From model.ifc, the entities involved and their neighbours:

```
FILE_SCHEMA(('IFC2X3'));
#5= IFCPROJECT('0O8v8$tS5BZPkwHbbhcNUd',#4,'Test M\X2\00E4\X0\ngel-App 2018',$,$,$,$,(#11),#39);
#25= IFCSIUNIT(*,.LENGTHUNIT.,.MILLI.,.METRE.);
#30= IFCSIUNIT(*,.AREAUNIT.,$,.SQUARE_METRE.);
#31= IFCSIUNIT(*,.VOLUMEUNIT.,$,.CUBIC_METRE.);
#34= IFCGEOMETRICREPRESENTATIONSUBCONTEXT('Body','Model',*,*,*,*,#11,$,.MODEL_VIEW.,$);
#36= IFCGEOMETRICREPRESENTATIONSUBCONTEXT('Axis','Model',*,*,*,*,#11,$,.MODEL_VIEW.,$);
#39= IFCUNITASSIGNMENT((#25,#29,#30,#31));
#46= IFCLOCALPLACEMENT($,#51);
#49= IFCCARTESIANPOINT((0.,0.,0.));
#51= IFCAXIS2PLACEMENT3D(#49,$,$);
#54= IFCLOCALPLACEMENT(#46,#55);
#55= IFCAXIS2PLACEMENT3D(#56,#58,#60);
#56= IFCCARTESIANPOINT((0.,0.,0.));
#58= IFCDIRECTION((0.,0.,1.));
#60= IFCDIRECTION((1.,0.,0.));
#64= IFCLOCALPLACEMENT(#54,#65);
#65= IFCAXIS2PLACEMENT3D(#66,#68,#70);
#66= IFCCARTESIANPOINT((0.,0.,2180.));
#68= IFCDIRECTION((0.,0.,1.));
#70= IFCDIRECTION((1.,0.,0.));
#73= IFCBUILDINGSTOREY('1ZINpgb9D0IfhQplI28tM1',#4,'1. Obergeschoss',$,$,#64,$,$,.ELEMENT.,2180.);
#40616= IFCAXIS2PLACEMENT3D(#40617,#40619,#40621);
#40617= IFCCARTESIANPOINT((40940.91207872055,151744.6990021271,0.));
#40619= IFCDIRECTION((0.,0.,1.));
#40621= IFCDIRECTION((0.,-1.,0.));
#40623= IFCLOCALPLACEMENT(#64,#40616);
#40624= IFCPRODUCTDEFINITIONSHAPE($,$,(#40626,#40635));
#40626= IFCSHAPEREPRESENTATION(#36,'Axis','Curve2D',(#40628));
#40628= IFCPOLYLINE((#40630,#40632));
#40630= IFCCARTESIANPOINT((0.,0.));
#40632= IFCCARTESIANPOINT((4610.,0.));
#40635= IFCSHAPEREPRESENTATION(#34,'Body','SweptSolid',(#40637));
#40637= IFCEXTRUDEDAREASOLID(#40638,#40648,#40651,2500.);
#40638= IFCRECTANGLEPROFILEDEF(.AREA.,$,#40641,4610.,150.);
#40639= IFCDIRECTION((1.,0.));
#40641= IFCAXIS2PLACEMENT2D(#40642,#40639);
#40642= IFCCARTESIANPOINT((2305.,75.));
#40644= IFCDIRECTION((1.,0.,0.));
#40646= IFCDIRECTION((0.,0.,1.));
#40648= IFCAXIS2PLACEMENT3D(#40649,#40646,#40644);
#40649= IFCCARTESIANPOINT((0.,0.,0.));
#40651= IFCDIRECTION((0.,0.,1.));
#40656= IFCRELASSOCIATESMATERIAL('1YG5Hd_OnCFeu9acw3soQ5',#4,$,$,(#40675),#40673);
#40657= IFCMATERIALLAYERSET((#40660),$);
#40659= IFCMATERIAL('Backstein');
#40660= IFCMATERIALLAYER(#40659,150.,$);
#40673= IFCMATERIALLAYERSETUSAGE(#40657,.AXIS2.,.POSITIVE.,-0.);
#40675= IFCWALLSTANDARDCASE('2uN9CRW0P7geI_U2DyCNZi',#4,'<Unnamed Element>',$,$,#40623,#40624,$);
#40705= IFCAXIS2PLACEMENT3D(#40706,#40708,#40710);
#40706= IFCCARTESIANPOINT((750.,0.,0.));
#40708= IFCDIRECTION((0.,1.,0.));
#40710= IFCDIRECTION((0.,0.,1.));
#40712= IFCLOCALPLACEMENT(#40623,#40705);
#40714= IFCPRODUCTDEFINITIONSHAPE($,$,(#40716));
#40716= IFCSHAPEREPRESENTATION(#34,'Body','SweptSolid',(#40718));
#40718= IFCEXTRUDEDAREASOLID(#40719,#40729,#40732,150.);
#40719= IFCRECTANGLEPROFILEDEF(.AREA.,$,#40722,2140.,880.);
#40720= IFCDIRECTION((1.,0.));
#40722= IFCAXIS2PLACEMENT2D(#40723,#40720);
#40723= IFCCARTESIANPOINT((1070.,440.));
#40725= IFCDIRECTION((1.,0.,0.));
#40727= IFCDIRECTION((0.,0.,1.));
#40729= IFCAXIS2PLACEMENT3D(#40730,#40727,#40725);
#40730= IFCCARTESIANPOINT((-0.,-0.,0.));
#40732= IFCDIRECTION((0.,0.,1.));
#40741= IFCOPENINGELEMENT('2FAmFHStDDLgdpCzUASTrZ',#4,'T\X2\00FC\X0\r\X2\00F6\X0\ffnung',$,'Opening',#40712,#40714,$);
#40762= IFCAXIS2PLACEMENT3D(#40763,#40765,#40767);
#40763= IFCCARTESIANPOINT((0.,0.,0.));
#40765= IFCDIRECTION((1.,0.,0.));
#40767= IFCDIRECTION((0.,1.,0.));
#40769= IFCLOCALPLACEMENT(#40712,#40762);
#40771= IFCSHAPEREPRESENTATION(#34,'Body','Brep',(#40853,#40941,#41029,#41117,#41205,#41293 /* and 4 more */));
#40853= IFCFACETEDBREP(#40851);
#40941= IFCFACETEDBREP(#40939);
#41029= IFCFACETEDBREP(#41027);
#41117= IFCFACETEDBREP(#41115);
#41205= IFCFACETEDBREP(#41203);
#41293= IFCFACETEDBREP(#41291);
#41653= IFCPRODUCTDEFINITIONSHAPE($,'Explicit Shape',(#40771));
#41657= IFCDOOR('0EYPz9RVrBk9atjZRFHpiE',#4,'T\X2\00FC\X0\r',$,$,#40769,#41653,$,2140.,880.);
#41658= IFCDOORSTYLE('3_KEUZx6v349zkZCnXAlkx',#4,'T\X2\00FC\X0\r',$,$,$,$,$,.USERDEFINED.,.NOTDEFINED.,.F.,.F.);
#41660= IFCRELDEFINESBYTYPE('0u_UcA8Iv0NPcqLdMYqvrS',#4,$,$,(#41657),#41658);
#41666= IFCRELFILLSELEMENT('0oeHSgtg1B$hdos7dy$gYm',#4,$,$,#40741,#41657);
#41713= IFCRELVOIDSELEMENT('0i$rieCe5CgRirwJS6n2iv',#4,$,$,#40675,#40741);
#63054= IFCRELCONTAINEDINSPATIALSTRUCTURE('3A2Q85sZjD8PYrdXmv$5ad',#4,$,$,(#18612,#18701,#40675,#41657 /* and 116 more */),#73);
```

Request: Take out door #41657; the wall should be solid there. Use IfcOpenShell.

```python
import ifcopenshell
import ifcopenshell.api.feature
import ifcopenshell.api.root
import ifcopenshell.geom
import ifcopenshell.util.shape

model = ifcopenshell.open("model.ifc")
settings = ifcopenshell.geom.settings()


def volume(element):
    """Net volume in cubic metres, openings subtracted."""
    shape = ifcopenshell.geom.create_shape(settings, element)
    return ifcopenshell.util.shape.get_volume(shape.geometry)


door = model.by_guid("0EYPz9RVrBk9atjZRFHpiE")
opening = door.FillsVoids[0].RelatingOpeningElement
wall = opening.VoidsElements[0].RelatingBuildingElement
before = volume(wall)

ifcopenshell.api.root.remove_product(model, product=door)
ifcopenshell.api.feature.remove_feature(model, feature=opening)

after = volume(wall)

print(f"wall volume {before:.3f} -> {after:.3f} m3")

model.write("model_edited.ifc")
```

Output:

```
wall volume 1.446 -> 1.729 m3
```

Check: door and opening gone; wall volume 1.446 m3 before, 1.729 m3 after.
